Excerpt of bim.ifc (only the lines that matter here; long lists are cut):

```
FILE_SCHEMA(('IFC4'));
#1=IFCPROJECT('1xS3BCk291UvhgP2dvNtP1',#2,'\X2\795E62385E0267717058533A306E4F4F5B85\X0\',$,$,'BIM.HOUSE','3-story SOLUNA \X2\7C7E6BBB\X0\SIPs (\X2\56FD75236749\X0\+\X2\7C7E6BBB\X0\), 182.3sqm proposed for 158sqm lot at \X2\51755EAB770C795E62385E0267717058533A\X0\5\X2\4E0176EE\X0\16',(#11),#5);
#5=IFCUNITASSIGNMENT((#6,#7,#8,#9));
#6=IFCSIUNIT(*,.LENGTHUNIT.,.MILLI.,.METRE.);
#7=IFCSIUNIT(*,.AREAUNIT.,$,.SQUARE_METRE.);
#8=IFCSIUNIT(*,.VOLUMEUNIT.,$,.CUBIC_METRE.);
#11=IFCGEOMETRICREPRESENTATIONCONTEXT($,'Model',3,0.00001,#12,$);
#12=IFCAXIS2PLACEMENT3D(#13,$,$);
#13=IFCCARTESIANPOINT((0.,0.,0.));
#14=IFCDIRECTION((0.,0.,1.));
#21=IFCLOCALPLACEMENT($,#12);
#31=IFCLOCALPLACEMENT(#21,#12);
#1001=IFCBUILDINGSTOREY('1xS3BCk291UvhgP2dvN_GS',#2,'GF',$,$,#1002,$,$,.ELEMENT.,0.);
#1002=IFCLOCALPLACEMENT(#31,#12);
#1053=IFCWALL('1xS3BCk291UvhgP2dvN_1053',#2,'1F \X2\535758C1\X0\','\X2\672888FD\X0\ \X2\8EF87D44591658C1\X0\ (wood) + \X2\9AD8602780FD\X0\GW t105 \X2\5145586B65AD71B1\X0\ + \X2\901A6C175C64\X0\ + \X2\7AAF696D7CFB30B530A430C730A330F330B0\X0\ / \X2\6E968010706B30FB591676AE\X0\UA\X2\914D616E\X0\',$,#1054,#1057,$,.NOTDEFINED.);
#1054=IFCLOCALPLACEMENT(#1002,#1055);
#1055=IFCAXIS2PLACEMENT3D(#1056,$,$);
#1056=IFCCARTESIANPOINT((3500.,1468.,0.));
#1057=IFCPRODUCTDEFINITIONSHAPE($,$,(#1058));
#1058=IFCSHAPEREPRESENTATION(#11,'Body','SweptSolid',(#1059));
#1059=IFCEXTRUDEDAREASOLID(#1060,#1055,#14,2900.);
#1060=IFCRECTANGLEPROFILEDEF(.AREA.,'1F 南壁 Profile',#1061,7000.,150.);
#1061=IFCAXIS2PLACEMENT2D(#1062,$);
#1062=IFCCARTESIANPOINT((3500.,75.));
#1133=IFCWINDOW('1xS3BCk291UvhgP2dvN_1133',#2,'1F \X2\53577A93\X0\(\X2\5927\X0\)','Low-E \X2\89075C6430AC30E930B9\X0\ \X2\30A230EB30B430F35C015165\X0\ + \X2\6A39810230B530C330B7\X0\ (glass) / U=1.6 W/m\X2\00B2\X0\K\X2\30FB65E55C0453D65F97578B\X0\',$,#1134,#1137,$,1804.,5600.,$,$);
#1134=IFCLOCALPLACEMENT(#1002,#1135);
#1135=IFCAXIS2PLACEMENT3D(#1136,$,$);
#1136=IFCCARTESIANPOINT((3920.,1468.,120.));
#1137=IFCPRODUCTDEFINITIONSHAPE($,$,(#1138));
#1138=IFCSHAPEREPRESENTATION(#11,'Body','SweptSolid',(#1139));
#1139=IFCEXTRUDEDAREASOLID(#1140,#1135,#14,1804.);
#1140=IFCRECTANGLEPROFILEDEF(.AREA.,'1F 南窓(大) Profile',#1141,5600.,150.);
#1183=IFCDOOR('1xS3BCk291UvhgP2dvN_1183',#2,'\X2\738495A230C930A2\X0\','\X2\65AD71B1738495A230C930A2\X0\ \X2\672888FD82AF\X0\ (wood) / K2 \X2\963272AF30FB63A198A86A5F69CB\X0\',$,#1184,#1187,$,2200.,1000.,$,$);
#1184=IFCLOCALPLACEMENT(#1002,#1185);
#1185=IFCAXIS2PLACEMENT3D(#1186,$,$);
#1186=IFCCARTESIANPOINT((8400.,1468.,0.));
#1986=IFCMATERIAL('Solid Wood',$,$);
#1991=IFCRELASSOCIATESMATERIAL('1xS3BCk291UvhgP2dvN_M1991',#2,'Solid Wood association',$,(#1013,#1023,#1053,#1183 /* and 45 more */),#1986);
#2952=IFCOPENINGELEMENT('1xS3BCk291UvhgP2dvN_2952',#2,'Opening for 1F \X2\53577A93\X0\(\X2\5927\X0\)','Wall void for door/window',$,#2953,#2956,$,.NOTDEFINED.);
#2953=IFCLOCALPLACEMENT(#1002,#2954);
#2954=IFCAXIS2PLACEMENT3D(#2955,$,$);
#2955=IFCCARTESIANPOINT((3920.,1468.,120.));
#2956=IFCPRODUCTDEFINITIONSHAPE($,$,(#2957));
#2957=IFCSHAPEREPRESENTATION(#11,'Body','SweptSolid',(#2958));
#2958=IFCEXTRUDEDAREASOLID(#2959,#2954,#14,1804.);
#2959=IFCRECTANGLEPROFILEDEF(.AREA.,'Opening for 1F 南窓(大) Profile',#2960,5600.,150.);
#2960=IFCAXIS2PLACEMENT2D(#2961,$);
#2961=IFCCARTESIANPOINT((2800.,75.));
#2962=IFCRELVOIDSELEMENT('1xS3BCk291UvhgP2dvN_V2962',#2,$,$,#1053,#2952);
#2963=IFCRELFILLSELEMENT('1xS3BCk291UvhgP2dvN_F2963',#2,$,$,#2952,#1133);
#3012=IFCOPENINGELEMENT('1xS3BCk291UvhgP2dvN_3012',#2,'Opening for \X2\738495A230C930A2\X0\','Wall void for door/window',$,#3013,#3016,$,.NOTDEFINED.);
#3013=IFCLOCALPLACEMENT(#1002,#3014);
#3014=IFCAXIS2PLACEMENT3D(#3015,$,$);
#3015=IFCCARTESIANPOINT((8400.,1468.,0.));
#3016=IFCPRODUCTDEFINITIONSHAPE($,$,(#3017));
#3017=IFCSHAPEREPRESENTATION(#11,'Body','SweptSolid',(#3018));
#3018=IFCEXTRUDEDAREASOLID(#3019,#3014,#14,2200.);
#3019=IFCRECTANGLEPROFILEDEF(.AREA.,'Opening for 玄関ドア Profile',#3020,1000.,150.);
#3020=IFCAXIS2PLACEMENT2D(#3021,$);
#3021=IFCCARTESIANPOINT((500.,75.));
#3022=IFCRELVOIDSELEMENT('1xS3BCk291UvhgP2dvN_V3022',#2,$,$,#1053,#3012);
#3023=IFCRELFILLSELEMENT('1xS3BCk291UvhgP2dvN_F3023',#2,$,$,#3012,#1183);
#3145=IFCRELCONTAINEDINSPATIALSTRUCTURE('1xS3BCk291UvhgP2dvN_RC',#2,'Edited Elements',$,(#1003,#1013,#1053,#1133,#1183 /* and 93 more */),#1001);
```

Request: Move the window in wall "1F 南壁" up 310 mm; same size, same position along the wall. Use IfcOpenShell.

```python
import numpy as np
import ifcopenshell
import ifcopenshell.api.geometry
import ifcopenshell.util.placement
import ifcopenshell.util.unit

model = ifcopenshell.open("bim.ifc")
unit_scale = ifcopenshell.util.unit.calculate_unit_scale(model)

window = model.by_guid("1xS3BCk291UvhgP2dvN_1133")
opening = window.FillsVoids[0].RelatingOpeningElement
dz = 0.31 / unit_scale

shift = np.array([0.0, 0.0, dz])
# The window is not placed relative to its opening, so move both.
for product in (opening, window):
    matrix = ifcopenshell.util.placement.get_local_placement(product.ObjectPlacement)
    matrix[:3, 3] += shift
    ifcopenshell.api.geometry.edit_object_placement(model, product=product, matrix=matrix, is_si=False)

print(f"moved by {dz * unit_scale:+.3f} m")

model.write("bim_updated.ifc")
```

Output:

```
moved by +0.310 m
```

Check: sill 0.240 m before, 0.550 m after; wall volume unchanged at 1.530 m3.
